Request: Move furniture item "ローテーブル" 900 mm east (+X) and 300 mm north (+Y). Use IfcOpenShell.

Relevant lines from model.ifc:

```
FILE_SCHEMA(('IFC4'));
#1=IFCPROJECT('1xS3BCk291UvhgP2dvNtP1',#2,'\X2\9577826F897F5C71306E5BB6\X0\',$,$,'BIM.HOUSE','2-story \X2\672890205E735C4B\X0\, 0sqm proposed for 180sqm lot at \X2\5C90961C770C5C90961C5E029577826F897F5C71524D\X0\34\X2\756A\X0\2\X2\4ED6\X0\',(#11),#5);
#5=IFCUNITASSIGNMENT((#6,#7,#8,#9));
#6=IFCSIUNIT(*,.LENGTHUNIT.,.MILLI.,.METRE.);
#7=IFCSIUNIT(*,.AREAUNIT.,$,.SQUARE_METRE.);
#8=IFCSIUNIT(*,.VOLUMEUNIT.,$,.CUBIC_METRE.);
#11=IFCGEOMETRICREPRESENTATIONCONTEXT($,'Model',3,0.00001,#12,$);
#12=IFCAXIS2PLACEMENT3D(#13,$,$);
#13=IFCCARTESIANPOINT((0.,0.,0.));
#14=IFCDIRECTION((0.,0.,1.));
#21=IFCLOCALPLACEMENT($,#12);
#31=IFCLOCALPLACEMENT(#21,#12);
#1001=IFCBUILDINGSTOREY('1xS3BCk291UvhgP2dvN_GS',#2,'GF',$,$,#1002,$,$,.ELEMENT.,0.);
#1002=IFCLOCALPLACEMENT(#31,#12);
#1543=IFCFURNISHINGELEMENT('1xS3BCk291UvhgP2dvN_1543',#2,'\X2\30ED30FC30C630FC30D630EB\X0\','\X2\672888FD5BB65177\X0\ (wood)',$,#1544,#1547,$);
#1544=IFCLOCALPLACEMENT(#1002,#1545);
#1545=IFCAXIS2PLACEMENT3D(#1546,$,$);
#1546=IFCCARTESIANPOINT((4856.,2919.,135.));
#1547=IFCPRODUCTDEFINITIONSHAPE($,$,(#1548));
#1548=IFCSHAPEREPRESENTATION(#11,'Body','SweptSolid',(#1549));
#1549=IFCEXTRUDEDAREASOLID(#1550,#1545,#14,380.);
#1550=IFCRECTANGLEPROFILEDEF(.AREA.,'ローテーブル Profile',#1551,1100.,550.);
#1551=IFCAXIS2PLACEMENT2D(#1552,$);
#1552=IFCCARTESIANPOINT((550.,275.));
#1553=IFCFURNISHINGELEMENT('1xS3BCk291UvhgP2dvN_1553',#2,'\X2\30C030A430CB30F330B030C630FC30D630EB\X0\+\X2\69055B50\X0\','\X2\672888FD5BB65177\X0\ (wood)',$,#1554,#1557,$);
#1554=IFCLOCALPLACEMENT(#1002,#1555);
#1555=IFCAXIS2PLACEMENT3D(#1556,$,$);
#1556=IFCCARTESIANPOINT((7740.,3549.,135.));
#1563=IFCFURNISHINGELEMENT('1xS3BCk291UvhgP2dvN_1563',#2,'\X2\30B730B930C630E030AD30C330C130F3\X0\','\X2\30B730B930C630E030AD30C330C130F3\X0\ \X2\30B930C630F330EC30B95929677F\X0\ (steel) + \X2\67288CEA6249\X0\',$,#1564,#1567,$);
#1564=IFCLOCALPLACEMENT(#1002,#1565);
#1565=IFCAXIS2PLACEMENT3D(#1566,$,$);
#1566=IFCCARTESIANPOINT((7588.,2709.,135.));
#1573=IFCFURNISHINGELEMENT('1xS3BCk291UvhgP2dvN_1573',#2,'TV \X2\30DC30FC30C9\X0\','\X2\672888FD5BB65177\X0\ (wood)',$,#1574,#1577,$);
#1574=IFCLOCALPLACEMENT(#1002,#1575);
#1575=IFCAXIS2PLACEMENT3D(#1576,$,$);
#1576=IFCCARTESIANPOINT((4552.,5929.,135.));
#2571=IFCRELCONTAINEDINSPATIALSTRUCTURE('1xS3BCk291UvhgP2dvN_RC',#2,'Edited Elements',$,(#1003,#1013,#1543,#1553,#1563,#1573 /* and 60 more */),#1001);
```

```python
import ifcopenshell
import ifcopenshell.api.geometry
import ifcopenshell.util.placement
import ifcopenshell.util.unit

model = ifcopenshell.open("model.ifc")
unit_scale = ifcopenshell.util.unit.calculate_unit_scale(model)

item = model.by_guid("1xS3BCk291UvhgP2dvN_1543")
matrix = ifcopenshell.util.placement.get_local_placement(item.ObjectPlacement)
matrix[0, 3] += 0.9 / unit_scale
matrix[1, 3] += 0.3 / unit_scale
ifcopenshell.api.geometry.edit_object_placement(model, product=item, matrix=matrix, is_si=False)

print(ifcopenshell.util.placement.get_local_placement(item.ObjectPlacement).round(3) + 0.0)

model.write("model_updated.ifc")
```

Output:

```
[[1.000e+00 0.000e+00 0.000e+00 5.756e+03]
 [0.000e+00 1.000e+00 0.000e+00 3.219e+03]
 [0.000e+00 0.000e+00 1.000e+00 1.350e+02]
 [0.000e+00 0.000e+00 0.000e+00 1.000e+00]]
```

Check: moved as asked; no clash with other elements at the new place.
